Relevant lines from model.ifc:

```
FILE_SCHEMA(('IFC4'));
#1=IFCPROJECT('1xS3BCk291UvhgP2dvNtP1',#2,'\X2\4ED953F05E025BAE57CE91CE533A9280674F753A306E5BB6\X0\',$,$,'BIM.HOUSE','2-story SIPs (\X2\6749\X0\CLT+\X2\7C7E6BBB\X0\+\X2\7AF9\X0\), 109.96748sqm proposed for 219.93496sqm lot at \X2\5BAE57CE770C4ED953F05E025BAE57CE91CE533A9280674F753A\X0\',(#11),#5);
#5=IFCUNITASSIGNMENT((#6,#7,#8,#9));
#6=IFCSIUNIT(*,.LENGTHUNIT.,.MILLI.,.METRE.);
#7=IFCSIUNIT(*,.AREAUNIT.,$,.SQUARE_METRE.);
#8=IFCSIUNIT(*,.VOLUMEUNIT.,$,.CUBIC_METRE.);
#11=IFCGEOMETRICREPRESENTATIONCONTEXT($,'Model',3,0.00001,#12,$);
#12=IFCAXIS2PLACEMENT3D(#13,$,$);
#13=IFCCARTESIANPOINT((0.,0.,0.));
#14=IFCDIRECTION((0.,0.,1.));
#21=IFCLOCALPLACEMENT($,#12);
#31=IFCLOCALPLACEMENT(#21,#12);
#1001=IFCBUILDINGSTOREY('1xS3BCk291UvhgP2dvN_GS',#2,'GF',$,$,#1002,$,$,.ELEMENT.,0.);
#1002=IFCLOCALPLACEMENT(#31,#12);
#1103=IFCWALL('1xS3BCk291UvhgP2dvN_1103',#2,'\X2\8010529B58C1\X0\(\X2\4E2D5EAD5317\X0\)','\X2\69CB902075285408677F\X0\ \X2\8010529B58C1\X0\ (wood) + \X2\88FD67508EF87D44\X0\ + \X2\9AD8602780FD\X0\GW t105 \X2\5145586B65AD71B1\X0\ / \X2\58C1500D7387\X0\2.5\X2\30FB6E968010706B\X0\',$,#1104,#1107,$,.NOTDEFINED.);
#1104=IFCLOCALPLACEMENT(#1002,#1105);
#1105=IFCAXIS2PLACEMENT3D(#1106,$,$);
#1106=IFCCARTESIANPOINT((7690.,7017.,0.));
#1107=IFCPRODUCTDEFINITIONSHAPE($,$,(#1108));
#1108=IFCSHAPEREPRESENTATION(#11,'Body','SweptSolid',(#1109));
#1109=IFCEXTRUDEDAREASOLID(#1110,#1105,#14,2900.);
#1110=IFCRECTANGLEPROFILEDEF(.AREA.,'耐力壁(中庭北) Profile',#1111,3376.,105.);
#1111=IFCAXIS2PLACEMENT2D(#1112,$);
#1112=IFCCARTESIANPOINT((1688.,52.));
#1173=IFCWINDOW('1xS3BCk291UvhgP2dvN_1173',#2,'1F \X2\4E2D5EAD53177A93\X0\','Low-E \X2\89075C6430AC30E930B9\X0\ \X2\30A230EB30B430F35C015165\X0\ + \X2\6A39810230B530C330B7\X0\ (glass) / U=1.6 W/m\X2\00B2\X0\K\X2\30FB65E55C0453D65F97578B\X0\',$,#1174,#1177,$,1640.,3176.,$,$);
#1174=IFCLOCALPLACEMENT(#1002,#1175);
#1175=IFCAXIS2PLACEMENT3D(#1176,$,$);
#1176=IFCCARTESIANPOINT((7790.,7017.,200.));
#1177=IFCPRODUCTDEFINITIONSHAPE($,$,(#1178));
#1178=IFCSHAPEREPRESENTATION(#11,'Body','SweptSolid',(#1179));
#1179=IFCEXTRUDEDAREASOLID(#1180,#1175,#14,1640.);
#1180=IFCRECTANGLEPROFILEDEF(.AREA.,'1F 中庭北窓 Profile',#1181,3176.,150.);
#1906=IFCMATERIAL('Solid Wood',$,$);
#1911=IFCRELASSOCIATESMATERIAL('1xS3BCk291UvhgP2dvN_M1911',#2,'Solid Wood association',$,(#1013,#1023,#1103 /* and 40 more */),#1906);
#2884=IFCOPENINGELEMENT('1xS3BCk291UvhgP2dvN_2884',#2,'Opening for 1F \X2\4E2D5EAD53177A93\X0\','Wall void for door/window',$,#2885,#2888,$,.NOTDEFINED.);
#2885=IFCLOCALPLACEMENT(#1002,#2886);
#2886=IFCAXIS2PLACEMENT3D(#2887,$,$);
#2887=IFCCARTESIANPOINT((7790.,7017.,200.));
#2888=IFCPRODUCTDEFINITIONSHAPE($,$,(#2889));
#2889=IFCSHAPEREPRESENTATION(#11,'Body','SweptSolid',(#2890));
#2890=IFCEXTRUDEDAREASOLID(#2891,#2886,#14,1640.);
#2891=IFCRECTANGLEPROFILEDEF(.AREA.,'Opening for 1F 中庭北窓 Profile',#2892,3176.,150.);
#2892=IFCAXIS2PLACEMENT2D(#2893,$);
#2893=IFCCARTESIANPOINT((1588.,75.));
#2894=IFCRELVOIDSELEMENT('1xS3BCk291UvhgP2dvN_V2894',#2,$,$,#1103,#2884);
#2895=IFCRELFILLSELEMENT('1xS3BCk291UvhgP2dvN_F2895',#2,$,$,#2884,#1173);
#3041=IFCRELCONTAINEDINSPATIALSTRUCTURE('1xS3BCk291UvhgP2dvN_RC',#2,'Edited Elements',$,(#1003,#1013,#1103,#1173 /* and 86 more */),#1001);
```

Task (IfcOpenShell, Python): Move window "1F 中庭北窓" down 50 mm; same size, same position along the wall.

```python
import numpy as np
import ifcopenshell
import ifcopenshell.api.geometry
import ifcopenshell.util.placement
import ifcopenshell.util.unit

model = ifcopenshell.open("model.ifc")
unit_scale = ifcopenshell.util.unit.calculate_unit_scale(model)

window = model.by_guid("1xS3BCk291UvhgP2dvN_1173")
opening = window.FillsVoids[0].RelatingOpeningElement
dz = -50.0

shift = np.array([0.0, 0.0, dz])
# The window is not placed relative to its opening, so move both.
for product in (opening, window):
    matrix = ifcopenshell.util.placement.get_local_placement(product.ObjectPlacement)
    matrix[:3, 3] += shift
    ifcopenshell.api.geometry.edit_object_placement(model, product=product, matrix=matrix, is_si=False)

print(f"moved by {dz * unit_scale:+.3f} m")

model.write("model_rev.ifc")
```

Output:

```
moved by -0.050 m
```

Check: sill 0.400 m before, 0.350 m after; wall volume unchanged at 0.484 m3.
